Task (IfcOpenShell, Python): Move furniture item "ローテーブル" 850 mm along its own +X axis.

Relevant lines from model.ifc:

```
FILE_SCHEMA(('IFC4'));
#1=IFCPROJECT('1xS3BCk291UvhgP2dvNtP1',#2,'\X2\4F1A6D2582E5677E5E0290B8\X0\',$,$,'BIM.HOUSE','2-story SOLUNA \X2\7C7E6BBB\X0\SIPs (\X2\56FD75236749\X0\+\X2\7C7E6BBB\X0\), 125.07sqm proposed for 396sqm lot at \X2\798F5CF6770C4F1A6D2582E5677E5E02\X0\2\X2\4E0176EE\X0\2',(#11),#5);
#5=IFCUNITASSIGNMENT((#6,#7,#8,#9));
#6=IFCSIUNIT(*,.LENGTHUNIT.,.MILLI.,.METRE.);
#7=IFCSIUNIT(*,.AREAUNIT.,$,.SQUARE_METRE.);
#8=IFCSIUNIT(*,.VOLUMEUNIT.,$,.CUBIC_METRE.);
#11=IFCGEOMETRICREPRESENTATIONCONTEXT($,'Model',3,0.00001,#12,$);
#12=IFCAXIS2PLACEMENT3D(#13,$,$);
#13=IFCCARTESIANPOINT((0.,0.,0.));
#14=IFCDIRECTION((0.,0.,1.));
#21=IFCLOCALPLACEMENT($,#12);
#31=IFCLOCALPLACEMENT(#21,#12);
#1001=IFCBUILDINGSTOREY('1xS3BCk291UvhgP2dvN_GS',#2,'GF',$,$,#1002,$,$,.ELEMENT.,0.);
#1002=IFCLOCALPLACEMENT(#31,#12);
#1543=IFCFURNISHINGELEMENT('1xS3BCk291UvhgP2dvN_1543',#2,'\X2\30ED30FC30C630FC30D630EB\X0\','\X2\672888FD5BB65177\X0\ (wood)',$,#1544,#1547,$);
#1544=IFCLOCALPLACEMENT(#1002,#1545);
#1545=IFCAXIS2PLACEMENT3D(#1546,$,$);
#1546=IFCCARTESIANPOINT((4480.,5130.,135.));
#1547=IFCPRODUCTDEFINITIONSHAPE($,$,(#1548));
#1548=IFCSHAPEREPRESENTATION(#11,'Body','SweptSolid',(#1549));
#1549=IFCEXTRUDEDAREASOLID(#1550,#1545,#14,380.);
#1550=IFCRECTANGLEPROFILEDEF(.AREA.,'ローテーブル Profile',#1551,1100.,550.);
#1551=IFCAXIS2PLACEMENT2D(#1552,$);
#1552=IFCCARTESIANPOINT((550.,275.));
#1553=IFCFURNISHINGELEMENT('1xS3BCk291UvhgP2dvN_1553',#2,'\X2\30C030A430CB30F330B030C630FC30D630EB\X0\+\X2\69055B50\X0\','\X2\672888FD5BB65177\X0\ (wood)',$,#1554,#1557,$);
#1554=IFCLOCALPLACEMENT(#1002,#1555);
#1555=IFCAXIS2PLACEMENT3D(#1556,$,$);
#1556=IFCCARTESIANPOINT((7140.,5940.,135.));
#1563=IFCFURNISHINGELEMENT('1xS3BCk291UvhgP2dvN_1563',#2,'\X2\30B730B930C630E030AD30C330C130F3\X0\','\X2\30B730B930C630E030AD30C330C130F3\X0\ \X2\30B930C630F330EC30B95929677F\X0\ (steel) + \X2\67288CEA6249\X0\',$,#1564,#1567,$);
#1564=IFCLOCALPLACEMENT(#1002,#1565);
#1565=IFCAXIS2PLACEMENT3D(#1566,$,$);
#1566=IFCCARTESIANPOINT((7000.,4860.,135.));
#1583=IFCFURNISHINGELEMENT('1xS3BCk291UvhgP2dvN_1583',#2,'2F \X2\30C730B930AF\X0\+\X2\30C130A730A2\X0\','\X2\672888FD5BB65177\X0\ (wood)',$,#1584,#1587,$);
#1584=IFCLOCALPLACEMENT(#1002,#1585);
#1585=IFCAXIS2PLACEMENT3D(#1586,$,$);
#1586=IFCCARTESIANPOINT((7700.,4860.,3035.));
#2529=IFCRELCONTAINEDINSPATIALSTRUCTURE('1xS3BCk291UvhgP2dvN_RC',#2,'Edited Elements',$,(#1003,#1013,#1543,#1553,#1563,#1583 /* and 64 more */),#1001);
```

```python
import ifcopenshell
import ifcopenshell.api.geometry
import ifcopenshell.util.placement
import ifcopenshell.util.unit

model = ifcopenshell.open("model.ifc")
unit_scale = ifcopenshell.util.unit.calculate_unit_scale(model)

item = model.by_id(1543)
matrix = ifcopenshell.util.placement.get_local_placement(item.ObjectPlacement)
matrix[:3, 3] += matrix[:3, 0] * 0.85 / unit_scale
ifcopenshell.api.geometry.edit_object_placement(model, product=item, matrix=matrix, is_si=False)

print(ifcopenshell.util.placement.get_local_placement(item.ObjectPlacement).round(3) + 0.0)

model.write("model_updated.ifc")
```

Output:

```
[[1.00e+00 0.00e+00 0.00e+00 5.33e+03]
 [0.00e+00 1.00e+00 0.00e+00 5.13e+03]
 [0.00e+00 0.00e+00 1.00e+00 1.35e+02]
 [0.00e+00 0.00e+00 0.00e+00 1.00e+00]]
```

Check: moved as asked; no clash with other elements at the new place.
